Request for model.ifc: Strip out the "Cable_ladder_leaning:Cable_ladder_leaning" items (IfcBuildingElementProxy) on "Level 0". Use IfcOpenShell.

First a look at what the model holds.

```python
import ifcopenshell
import ifcopenshell.util.element

model = ifcopenshell.open("model.ifc")
print(model.schema)
storey = next(s for s in model.by_type("IfcBuildingStorey") if s.Name == "Level 0")
proxies = [e for e in ifcopenshell.util.element.get_decomposition(storey) if e.is_a("IfcBuildingElementProxy")]
seen = {}
for e in proxies:
    element_type = ifcopenshell.util.element.get_type(e)
    name = element_type.Name if element_type not in (None, e) else None
    seen[name] = seen.get(name, 0) + 1
for name, count in sorted(seen.items(), key=str):
    print(count, "x", name)
```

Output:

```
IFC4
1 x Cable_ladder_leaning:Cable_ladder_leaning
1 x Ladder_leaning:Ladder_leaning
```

```python
import ifcopenshell
import ifcopenshell.api.root
import ifcopenshell.util.element

model = ifcopenshell.open("model.ifc")

storey = next(s for s in model.by_type("IfcBuildingStorey") if s.Name == "Level 0")
proxies = [e for e in ifcopenshell.util.element.get_decomposition(storey) if e.is_a("IfcBuildingElementProxy")]
targets = [e for e in proxies if (t := ifcopenshell.util.element.get_type(e)) not in (None, e) and t.Name == "Cable_ladder_leaning:Cable_ladder_leaning"]

for e in targets:
    ifcopenshell.api.root.remove_product(model, product=e)
print(len(targets), "removed")

model.write("model_v2.ifc")
```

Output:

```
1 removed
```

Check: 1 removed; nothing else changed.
